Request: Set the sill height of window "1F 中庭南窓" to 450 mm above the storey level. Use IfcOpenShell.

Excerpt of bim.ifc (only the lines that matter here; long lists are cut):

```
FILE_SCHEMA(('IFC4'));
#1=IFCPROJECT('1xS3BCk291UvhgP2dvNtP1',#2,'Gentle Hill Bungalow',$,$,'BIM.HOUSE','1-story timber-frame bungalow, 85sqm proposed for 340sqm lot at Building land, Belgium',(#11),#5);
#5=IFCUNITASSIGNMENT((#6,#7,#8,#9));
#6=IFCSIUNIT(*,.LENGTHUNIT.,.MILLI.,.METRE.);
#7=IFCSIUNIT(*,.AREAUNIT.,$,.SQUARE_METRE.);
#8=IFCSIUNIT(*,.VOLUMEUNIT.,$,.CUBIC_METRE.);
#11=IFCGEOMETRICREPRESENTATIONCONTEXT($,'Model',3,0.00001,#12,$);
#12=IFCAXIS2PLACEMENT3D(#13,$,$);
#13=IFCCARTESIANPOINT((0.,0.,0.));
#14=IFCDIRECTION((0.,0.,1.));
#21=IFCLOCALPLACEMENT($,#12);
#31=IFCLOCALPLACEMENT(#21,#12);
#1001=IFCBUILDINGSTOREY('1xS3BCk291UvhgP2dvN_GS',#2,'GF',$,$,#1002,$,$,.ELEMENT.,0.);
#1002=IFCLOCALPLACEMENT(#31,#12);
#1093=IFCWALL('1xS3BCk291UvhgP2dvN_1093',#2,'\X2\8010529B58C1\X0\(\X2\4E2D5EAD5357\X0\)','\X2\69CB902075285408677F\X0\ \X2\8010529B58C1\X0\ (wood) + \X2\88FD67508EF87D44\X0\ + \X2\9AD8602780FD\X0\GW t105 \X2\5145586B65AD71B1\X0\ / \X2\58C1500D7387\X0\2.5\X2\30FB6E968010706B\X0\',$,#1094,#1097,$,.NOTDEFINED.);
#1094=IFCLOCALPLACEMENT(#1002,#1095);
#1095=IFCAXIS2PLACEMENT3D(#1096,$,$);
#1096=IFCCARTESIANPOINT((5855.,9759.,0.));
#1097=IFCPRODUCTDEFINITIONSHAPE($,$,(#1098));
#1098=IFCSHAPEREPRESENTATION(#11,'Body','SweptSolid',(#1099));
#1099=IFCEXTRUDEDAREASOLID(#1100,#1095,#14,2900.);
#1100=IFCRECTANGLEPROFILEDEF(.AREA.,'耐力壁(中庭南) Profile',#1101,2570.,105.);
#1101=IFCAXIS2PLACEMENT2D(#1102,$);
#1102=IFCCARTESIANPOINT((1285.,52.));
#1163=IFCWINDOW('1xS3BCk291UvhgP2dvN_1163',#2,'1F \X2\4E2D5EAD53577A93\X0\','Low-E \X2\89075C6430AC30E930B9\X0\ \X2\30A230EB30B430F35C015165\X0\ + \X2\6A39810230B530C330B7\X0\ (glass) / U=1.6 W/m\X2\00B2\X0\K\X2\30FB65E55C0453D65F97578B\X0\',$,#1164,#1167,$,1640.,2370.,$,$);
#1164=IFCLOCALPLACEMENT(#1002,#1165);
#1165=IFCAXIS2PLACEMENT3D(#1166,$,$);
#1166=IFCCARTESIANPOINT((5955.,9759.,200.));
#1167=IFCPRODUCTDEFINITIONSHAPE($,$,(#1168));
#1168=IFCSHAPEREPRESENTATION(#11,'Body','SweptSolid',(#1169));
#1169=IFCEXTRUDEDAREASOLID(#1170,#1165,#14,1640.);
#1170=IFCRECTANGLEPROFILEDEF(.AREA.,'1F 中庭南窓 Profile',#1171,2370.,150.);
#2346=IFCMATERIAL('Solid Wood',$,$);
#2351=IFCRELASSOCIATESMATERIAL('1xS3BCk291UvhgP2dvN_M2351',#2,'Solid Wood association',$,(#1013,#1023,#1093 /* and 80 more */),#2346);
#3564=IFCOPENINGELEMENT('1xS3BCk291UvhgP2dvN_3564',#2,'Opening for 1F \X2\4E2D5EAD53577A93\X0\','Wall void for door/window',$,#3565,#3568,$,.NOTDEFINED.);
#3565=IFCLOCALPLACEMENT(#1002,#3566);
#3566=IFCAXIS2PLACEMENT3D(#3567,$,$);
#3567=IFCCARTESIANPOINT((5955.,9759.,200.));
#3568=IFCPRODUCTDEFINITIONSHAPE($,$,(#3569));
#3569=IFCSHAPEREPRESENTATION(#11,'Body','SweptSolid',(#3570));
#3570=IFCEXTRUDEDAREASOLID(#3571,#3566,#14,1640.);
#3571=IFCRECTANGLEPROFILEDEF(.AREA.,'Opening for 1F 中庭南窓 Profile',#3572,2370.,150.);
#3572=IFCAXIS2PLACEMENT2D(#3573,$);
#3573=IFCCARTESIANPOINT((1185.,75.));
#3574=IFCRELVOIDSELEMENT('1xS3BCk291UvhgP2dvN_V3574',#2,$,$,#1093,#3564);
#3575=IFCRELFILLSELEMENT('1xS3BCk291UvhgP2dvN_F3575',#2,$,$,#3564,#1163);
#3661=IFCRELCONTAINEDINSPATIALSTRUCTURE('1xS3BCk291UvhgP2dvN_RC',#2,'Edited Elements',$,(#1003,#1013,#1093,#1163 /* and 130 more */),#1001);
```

```python
import numpy as np
import ifcopenshell
import ifcopenshell.api.geometry
import ifcopenshell.geom
import ifcopenshell.util.element
import ifcopenshell.util.placement
import ifcopenshell.util.shape
import ifcopenshell.util.unit

model = ifcopenshell.open("bim.ifc")
unit_scale = ifcopenshell.util.unit.calculate_unit_scale(model)

window = model.by_guid("1xS3BCk291UvhgP2dvN_1163")
opening = window.FillsVoids[0].RelatingOpeningElement
storey = ifcopenshell.util.element.get_container(window, ifc_class="IfcBuildingStorey")
level = ifcopenshell.util.placement.get_local_placement(storey.ObjectPlacement)[2, 3]

# The opening's origin need not be at the sill, so measure its lowest point.
shape = ifcopenshell.geom.create_shape(ifcopenshell.geom.settings(), opening)
bottom = ifcopenshell.util.shape.get_shape_bottom_elevation(shape, shape.geometry) / unit_scale
dz = level + 0.45 / unit_scale - bottom

shift = np.array([0.0, 0.0, dz])
# The window is not placed relative to its opening, so move both.
for product in (opening, window):
    matrix = ifcopenshell.util.placement.get_local_placement(product.ObjectPlacement)
    matrix[:3, 3] += shift
    ifcopenshell.api.geometry.edit_object_placement(model, product=product, matrix=matrix, is_si=False)

print(f"moved by {dz * unit_scale:+.3f} m")

model.write("bim_v2.ifc")
```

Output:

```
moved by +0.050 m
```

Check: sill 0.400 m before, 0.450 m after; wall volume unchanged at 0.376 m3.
